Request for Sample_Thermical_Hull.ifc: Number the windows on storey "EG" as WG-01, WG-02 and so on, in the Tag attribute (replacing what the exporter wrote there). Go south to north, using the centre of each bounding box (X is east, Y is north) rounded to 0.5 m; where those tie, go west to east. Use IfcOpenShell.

First a look at what the model holds.

```python
import ifcopenshell
import ifcopenshell.util.element
import ifcopenshell.util.placement

model = ifcopenshell.open("Sample_Thermical_Hull.ifc")
print(model.schema)
storey = next(s for s in model.by_type("IfcBuildingStorey") if s.Name == "EG")
windows = [e for e in ifcopenshell.util.element.get_decomposition(storey) if e.is_a("IfcWindow")]
for e in sorted(windows, key=lambda e: e.id()):
    origin = ifcopenshell.util.placement.get_local_placement(e.ObjectPlacement)[:3, 3]
    print(e.id(), e.Tag, e.Name, origin.round(2) + 0.0, sep=" | ")
```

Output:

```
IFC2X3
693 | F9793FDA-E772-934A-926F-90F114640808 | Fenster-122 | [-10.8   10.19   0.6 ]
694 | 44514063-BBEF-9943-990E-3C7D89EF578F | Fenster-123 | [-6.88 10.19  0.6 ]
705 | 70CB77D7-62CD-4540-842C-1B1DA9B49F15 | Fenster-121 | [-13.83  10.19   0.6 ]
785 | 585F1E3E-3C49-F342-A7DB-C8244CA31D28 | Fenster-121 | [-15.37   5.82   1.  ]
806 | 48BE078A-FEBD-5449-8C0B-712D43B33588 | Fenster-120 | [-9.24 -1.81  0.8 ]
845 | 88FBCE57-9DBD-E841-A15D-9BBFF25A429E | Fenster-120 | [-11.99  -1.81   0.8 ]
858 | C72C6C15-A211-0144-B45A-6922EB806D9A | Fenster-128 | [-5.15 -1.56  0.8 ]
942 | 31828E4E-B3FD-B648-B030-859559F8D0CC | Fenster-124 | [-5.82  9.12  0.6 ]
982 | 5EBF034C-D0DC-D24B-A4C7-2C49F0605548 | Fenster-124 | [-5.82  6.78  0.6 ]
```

```python
import ifcopenshell
import ifcopenshell.geom
import ifcopenshell.util.element
import ifcopenshell.util.shape

model = ifcopenshell.open("Sample_Thermical_Hull.ifc")
settings = ifcopenshell.geom.settings()
settings.set("use-world-coords", True)


def centre(element):
    shape = ifcopenshell.geom.create_shape(settings, element)
    return ifcopenshell.util.shape.get_bbox_centroid(shape.geometry)


storey = next(s for s in model.by_type("IfcBuildingStorey") if s.Name == "EG")
windows = [e for e in ifcopenshell.util.element.get_decomposition(storey) if e.is_a("IfcWindow")]

# Insertion points can sit at a corner or the storey origin, so sort by the geometry (in metres).
centres = {e: centre(e) for e in windows}
windows.sort(key=lambda e: (round(centres[e][1] / 0.5), centres[e][0]))

for i, e in enumerate(windows, start=1):
    number = f"WG-{i:02d}"
    e.Tag = number
    print(e.id(), number)

model.write("Sample_Thermical_Hull_rev.ifc")
```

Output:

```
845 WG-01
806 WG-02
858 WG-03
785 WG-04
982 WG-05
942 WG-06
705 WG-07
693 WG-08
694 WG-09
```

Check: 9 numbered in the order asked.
